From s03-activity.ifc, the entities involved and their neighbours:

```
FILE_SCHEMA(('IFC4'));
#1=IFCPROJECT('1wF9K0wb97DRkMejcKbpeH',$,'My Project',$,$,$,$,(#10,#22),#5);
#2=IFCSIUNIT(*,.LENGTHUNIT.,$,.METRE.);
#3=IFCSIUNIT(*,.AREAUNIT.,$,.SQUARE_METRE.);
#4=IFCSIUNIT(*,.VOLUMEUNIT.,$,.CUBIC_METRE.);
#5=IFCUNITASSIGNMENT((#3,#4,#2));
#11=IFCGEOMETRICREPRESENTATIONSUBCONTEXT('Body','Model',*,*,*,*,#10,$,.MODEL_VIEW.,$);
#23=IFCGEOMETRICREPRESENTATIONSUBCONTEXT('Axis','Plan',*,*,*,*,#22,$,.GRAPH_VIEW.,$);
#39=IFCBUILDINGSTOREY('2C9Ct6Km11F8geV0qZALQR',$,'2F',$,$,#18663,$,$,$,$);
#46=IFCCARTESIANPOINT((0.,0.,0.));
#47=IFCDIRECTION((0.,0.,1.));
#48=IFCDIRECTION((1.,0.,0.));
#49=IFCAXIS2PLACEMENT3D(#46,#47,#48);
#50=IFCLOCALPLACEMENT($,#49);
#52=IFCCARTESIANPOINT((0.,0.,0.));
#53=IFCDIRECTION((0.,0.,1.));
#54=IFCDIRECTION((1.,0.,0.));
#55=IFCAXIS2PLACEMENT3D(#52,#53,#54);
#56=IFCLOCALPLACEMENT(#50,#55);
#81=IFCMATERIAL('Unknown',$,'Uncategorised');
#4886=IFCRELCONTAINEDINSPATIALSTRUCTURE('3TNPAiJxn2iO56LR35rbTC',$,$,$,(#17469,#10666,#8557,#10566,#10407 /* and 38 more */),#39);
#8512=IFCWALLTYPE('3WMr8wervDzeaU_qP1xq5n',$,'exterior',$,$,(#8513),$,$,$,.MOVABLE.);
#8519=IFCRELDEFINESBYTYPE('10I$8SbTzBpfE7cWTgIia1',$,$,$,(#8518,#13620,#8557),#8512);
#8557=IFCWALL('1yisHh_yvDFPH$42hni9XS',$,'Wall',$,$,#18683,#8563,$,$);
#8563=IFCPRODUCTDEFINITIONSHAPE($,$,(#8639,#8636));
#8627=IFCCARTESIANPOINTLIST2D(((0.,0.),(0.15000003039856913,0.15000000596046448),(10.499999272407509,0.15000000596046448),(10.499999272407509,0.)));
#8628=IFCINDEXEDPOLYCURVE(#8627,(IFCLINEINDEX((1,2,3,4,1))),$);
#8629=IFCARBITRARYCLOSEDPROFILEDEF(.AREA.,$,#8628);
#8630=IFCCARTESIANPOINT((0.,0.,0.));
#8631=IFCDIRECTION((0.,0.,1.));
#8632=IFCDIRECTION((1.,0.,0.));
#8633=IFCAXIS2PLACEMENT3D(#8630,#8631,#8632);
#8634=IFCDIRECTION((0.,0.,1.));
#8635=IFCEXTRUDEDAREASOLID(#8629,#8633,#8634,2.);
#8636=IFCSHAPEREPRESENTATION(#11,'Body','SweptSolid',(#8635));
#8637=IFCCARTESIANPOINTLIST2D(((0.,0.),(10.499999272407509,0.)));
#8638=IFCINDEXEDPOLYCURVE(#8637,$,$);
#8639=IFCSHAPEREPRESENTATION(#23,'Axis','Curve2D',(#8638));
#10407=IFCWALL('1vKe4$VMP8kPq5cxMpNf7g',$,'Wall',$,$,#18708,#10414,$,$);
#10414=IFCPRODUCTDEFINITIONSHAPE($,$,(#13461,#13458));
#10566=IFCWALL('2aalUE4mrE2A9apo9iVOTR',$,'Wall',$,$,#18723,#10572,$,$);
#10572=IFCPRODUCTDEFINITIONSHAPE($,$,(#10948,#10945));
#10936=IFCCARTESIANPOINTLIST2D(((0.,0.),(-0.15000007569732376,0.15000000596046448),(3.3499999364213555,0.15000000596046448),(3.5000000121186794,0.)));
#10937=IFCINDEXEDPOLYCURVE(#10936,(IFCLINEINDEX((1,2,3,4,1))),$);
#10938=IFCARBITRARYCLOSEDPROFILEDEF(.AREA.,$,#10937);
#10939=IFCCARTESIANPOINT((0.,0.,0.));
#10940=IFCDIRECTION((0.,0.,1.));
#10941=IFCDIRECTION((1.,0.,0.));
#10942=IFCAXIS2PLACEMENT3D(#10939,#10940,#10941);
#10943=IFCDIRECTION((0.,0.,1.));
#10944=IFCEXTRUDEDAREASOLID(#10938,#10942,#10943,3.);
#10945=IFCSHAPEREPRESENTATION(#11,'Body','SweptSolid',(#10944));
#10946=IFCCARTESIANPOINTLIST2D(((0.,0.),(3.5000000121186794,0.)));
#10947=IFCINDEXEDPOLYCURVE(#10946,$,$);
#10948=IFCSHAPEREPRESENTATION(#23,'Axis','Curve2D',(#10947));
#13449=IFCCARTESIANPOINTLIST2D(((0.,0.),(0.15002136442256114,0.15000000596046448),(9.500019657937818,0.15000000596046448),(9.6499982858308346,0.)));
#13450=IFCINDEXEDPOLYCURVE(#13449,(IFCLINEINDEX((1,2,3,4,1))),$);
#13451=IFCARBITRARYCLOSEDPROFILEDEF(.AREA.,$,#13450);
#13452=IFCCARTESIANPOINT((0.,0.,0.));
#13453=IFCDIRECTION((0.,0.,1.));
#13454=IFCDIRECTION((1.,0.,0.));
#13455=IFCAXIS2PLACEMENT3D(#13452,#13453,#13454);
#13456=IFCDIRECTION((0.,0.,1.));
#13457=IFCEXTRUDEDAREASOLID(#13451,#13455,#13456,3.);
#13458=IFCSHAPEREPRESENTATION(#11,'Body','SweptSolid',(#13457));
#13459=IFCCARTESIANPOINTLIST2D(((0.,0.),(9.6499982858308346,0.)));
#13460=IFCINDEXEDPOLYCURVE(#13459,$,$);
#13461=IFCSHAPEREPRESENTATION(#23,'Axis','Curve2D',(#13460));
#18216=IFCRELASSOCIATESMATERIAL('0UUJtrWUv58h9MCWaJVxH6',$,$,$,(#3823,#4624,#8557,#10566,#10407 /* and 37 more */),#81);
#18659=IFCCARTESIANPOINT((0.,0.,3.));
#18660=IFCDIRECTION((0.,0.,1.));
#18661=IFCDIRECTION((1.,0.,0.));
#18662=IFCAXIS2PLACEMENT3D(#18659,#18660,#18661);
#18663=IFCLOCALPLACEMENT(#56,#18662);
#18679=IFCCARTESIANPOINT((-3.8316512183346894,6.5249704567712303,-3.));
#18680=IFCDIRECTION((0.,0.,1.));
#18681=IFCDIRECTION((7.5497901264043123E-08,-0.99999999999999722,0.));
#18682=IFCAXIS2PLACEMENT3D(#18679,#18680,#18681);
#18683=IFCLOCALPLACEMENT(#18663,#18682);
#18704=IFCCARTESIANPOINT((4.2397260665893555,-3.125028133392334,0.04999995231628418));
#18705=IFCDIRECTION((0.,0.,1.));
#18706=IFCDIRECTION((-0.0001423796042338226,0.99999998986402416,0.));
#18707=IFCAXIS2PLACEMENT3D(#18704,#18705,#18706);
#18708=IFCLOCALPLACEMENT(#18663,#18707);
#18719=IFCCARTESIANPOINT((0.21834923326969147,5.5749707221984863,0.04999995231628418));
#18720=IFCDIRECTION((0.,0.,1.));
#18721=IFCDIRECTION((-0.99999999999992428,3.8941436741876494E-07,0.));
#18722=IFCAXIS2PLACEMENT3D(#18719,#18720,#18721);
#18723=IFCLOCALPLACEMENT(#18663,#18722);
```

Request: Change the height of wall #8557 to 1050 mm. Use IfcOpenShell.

```python
import ifcopenshell
import ifcopenshell.geom
import ifcopenshell.util.representation
import ifcopenshell.util.shape

model = ifcopenshell.open("s03-activity.ifc")
settings = ifcopenshell.geom.settings()


def volume(element):
    """Net volume in cubic metres, openings subtracted."""
    shape = ifcopenshell.geom.create_shape(settings, element)
    return ifcopenshell.util.shape.get_volume(shape.geometry)


wall = model.by_guid("1yisHh_yvDFPH$42hni9XS")
before = volume(wall)

body = ifcopenshell.util.representation.get_representation(wall, "Model", "Body")
solid = body.Items[0]
old_height = solid.Depth
solid.Depth = 1.05
after = volume(wall)

print(f"height {old_height:g} -> {solid.Depth:g}, volume {before:.3f} -> {after:.3f} m3")

model.write("s03-activity_edited.ifc")
```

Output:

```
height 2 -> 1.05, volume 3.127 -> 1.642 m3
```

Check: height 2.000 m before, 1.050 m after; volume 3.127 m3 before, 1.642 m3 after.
